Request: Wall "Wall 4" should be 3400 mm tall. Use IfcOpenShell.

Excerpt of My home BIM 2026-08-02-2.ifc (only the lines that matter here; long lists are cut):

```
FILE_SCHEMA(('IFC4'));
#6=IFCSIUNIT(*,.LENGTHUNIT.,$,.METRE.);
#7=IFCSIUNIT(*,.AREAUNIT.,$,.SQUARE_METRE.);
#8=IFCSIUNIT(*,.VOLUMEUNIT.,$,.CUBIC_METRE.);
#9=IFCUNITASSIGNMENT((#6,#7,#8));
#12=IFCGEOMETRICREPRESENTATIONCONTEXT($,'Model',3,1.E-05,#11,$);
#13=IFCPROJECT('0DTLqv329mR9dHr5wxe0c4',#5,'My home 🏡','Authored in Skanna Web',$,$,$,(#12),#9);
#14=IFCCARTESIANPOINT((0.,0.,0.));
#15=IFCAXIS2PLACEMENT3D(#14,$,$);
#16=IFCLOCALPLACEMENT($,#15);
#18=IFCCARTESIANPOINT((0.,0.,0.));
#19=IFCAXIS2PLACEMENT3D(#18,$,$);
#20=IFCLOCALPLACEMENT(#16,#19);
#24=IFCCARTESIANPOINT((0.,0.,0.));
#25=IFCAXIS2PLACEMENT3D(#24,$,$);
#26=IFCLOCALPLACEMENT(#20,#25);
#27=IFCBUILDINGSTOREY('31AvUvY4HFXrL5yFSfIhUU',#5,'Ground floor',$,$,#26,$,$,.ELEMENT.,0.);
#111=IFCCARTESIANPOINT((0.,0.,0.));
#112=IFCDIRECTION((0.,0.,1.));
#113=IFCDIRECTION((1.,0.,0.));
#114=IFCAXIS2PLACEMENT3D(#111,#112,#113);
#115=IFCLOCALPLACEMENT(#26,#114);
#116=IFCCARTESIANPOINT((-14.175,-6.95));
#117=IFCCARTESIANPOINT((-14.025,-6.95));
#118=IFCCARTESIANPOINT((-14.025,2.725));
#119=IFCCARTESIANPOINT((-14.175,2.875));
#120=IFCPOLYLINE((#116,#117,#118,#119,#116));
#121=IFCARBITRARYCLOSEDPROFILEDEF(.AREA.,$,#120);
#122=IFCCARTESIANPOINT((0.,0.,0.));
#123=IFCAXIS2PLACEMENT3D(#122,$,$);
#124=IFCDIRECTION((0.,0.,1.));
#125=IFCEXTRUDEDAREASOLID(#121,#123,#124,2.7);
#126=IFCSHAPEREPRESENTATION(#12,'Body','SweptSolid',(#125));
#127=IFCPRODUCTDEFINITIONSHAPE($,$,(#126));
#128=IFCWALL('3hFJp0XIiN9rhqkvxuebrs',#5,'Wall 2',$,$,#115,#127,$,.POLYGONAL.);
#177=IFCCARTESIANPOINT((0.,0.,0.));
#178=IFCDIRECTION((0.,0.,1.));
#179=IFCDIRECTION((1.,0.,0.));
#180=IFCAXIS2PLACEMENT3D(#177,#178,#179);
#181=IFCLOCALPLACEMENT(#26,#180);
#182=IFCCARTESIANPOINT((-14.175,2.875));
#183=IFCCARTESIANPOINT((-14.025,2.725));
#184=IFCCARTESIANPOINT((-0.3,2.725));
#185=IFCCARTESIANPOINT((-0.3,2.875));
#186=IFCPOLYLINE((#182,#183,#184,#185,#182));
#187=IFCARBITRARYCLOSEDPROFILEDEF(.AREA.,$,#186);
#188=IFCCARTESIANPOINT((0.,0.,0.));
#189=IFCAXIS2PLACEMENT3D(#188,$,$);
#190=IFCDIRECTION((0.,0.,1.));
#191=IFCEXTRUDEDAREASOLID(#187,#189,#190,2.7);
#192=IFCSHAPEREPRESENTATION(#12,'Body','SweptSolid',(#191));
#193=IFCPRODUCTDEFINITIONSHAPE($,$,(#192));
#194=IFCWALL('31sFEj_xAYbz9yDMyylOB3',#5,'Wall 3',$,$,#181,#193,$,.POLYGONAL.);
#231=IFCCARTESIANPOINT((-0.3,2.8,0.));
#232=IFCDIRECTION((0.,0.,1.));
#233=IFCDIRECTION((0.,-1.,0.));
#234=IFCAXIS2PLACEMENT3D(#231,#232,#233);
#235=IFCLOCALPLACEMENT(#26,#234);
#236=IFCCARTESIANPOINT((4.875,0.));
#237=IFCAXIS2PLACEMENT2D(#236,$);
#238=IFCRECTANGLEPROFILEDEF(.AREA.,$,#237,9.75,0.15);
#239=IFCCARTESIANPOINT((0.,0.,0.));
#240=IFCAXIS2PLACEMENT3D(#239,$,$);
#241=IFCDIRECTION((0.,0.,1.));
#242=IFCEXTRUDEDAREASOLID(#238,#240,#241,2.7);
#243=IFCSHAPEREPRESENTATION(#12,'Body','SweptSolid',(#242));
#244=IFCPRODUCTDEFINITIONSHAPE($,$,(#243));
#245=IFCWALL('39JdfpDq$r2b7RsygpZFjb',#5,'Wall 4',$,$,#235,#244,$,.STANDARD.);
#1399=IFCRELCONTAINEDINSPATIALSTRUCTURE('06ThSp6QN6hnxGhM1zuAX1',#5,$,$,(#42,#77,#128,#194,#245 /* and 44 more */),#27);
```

```python
import ifcopenshell
import ifcopenshell.geom
import ifcopenshell.util.shape
import ifcopenshell.util.unit

model = ifcopenshell.open("My home BIM 2026-08-02-2.ifc")
unit_scale = ifcopenshell.util.unit.calculate_unit_scale(model)
settings = ifcopenshell.geom.settings()


def volume(element):
    """Net volume in cubic metres, openings subtracted."""
    shape = ifcopenshell.geom.create_shape(settings, element)
    return ifcopenshell.util.shape.get_volume(shape.geometry)


wall = model.by_guid("39JdfpDq$r2b7RsygpZFjb")
before = volume(wall)

body = next(r for r in wall.Representation.Representations if r.RepresentationIdentifier == "Body")
solid = body.Items[0]
old_height = solid.Depth
solid.Depth = 3.4 / unit_scale
after = volume(wall)

print(f"height {old_height:g} -> {solid.Depth:g}, volume {before:.3f} -> {after:.3f} m3")

model.write("My home BIM 2026-08-02-2_updated.ifc")
```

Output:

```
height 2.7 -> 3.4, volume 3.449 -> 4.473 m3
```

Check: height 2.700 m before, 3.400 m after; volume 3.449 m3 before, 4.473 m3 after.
